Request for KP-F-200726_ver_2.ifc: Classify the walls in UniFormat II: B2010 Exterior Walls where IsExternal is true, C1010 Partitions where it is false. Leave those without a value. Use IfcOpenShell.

First a look at what the model holds.

```python
import ifcopenshell
import ifcopenshell.util.element

model = ifcopenshell.open("KP-F-200726_ver_2.ifc")
print(model.schema)
print("classifications:", [c.Name for c in model.by_type("IfcClassification")])
values = [ifcopenshell.util.element.get_pset(e, "Pset_WallCommon", "IsExternal") for e in model.by_type("IfcWall")]
for value in (True, False, None):
    print("IsExternal", value, values.count(value))
```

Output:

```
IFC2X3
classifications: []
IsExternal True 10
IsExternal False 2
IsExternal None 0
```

```python
import ifcopenshell
import ifcopenshell.api.classification
import ifcopenshell.util.element

model = ifcopenshell.open("KP-F-200726_ver_2.ifc")

# IFC2X3 requires Source and Edition and has no link from the project to the system.
system = model.create_entity("IfcClassification", Source="ASTM", Edition="E1557", Name="UniFormat II")

walls = model.by_type("IfcWall")
external = {e: ifcopenshell.util.element.get_pset(e, "Pset_WallCommon", "IsExternal") for e in walls}
for flag, code, name in ((True, "B2010", "Exterior Walls"), (False, "C1010", "Partitions")):
    products = [e for e in walls if external[e] is flag]
    ifcopenshell.api.classification.add_reference(
        model, products=products, classification=system, identification=code, name=name
    )
    print(code, len(products))

model.write("KP-F-200726_ver_2-out.ifc")
```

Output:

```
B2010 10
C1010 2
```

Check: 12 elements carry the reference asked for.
